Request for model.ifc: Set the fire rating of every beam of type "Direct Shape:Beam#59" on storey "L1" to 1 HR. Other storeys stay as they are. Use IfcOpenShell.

First a look at what the model holds.

```python
import ifcopenshell
import ifcopenshell.util.element

model = ifcopenshell.open("model.ifc")
print(model.schema)
storey = next(s for s in model.by_type("IfcBuildingStorey") if s.Name == "L1")
beams = [e for e in ifcopenshell.util.element.get_decomposition(storey) if e.is_a("IfcBeam")]
seen = {}
for e in beams:
    element_type = ifcopenshell.util.element.get_type(e)
    key = (element_type.Name if element_type != e and element_type else None, ifcopenshell.util.element.get_pset(e, "Pset_BeamCommon", "FireRating"))
    seen[key] = seen.get(key, 0) + 1
for (name, value), count in sorted(seen.items(), key=str):
    print(count, "x", name, "|", value)
```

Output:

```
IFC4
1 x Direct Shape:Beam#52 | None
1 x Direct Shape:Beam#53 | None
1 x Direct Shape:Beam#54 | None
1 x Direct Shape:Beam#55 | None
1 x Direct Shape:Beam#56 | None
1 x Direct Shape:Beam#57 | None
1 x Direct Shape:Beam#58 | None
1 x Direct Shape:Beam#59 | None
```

```python
import ifcopenshell
import ifcopenshell.api.pset
import ifcopenshell.util.element

model = ifcopenshell.open("model.ifc")

storey = next(s for s in model.by_type("IfcBuildingStorey") if s.Name == "L1")
beams = [e for e in ifcopenshell.util.element.get_decomposition(storey) if e.is_a("IfcBeam")]

count = 0
for e in beams:
    element_type = ifcopenshell.util.element.get_type(e)
    if element_type in (None, e) or element_type.Name != "Direct Shape:Beam#59":
        continue
    # add_pset returns the element's existing set when there is one.
    pset = ifcopenshell.api.pset.add_pset(model, product=e, name="Pset_BeamCommon")
    ifcopenshell.api.pset.edit_pset(model, pset=pset, properties={"FireRating": "1 HR"})
    count += 1

print(count, "beams updated")

model.write("model_v2.ifc")
```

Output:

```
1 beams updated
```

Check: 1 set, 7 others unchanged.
